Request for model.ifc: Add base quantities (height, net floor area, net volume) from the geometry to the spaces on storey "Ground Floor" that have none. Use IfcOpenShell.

First a look at what the model holds.

```python
import ifcopenshell
import ifcopenshell.util.element
import ifcopenshell.util.unit

model = ifcopenshell.open("model.ifc")
print(model.schema)
for unit_type in ("LENGTHUNIT", "AREAUNIT", "VOLUMEUNIT"):
    print(unit_type, ifcopenshell.util.unit.calculate_unit_scale(model, unit_type))
storey = next(s for s in model.by_type("IfcBuildingStorey") if s.Name == "Ground Floor")
spaces = [e for e in ifcopenshell.util.element.get_decomposition(storey) if e.is_a("IfcSpace")]
for e in sorted(spaces, key=lambda e: e.id()):
    print(e.id(), e.is_a(), e.Name, list(ifcopenshell.util.element.get_psets(e, qtos_only=True)), sep=" | ")
```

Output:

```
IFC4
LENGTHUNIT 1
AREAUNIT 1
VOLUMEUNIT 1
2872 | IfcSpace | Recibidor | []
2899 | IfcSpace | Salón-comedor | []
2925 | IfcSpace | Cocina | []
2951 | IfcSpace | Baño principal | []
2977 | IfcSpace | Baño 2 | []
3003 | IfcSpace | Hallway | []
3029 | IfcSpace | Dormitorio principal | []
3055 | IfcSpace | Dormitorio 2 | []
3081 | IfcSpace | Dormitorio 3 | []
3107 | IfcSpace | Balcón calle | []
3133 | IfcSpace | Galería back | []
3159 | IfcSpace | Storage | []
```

```python
import ifcopenshell
import ifcopenshell.api.pset
import ifcopenshell.geom
import ifcopenshell.util.element
import ifcopenshell.util.shape
import ifcopenshell.util.unit

model = ifcopenshell.open("model.ifc")
unit_scale = ifcopenshell.util.unit.calculate_unit_scale(model)
area_scale = ifcopenshell.util.unit.calculate_unit_scale(model, "AREAUNIT")
volume_scale = ifcopenshell.util.unit.calculate_unit_scale(model, "VOLUMEUNIT")
settings = ifcopenshell.geom.settings()

storey = next(s for s in model.by_type("IfcBuildingStorey") if s.Name == "Ground Floor")
spaces = [e for e in ifcopenshell.util.element.get_decomposition(storey) if e.is_a("IfcSpace")]

for e in sorted(spaces, key=lambda e: e.id()):
    if ifcopenshell.util.element.get_psets(e, qtos_only=True, should_inherit=False):
        continue
    # Geometry comes back in metres, in the element's own axes.
    shape = ifcopenshell.geom.create_shape(settings, e)
    values = {
        "Height": ifcopenshell.util.shape.get_z(shape.geometry) / unit_scale,
        "NetFloorArea": ifcopenshell.util.shape.get_footprint_area(shape.geometry) / area_scale,
        "NetVolume": ifcopenshell.util.shape.get_volume(shape.geometry) / volume_scale,
    }
    qto = ifcopenshell.api.pset.add_qto(model, product=e, name="Qto_SpaceBaseQuantities")
    ifcopenshell.api.pset.edit_qto(model, qto=qto, properties=values)
    print(e.id(), {k: round(v, 3) for k, v in values.items()})

model.write("model_rev.ifc")
```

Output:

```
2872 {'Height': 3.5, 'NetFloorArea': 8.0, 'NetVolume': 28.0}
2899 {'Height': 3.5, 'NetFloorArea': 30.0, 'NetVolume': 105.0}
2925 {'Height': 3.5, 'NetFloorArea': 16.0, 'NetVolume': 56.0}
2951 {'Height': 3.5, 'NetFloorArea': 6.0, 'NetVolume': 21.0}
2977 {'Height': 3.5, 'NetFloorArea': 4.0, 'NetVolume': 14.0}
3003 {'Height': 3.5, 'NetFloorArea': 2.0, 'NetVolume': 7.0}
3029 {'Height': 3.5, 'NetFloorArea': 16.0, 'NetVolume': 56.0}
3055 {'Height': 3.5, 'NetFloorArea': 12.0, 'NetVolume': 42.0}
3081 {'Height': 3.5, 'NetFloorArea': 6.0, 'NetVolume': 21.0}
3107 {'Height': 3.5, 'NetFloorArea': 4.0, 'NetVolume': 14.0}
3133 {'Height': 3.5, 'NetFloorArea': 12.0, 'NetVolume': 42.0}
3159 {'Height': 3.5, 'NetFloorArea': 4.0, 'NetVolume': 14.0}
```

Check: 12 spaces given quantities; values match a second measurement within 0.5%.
